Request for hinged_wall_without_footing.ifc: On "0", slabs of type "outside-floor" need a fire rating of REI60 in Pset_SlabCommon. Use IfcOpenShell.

First a look at what the model holds.

```python
import ifcopenshell
import ifcopenshell.util.element

model = ifcopenshell.open("hinged_wall_without_footing.ifc")
print(model.schema)
storey = next(s for s in model.by_type("IfcBuildingStorey") if s.Name == "0")
slabs = [e for e in ifcopenshell.util.element.get_decomposition(storey) if e.is_a("IfcSlab")]
seen = {}
for e in slabs:
    element_type = ifcopenshell.util.element.get_type(e)
    key = (element_type.Name if element_type != e and element_type else None, ifcopenshell.util.element.get_pset(e, "Pset_SlabCommon", "FireRating"))
    seen[key] = seen.get(key, 0) + 1
for (name, value), count in sorted(seen.items(), key=str):
    print(count, "x", name, "|", value)
```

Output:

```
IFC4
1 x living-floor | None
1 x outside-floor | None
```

```python
import ifcopenshell
import ifcopenshell.api.pset
import ifcopenshell.util.element

model = ifcopenshell.open("hinged_wall_without_footing.ifc")

storey = next(s for s in model.by_type("IfcBuildingStorey") if s.Name == "0")
slabs = [e for e in ifcopenshell.util.element.get_decomposition(storey) if e.is_a("IfcSlab")]

count = 0
for e in slabs:
    element_type = ifcopenshell.util.element.get_type(e)
    if element_type in (None, e) or element_type.Name != "outside-floor":
        continue
    # add_pset returns the element's existing set when there is one.
    pset = ifcopenshell.api.pset.add_pset(model, product=e, name="Pset_SlabCommon")
    ifcopenshell.api.pset.edit_pset(model, pset=pset, properties={"FireRating": "REI60"})
    count += 1

print(count, "slabs updated")

model.write("hinged_wall_without_footing_rev.ifc")
```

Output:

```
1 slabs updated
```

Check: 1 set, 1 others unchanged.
